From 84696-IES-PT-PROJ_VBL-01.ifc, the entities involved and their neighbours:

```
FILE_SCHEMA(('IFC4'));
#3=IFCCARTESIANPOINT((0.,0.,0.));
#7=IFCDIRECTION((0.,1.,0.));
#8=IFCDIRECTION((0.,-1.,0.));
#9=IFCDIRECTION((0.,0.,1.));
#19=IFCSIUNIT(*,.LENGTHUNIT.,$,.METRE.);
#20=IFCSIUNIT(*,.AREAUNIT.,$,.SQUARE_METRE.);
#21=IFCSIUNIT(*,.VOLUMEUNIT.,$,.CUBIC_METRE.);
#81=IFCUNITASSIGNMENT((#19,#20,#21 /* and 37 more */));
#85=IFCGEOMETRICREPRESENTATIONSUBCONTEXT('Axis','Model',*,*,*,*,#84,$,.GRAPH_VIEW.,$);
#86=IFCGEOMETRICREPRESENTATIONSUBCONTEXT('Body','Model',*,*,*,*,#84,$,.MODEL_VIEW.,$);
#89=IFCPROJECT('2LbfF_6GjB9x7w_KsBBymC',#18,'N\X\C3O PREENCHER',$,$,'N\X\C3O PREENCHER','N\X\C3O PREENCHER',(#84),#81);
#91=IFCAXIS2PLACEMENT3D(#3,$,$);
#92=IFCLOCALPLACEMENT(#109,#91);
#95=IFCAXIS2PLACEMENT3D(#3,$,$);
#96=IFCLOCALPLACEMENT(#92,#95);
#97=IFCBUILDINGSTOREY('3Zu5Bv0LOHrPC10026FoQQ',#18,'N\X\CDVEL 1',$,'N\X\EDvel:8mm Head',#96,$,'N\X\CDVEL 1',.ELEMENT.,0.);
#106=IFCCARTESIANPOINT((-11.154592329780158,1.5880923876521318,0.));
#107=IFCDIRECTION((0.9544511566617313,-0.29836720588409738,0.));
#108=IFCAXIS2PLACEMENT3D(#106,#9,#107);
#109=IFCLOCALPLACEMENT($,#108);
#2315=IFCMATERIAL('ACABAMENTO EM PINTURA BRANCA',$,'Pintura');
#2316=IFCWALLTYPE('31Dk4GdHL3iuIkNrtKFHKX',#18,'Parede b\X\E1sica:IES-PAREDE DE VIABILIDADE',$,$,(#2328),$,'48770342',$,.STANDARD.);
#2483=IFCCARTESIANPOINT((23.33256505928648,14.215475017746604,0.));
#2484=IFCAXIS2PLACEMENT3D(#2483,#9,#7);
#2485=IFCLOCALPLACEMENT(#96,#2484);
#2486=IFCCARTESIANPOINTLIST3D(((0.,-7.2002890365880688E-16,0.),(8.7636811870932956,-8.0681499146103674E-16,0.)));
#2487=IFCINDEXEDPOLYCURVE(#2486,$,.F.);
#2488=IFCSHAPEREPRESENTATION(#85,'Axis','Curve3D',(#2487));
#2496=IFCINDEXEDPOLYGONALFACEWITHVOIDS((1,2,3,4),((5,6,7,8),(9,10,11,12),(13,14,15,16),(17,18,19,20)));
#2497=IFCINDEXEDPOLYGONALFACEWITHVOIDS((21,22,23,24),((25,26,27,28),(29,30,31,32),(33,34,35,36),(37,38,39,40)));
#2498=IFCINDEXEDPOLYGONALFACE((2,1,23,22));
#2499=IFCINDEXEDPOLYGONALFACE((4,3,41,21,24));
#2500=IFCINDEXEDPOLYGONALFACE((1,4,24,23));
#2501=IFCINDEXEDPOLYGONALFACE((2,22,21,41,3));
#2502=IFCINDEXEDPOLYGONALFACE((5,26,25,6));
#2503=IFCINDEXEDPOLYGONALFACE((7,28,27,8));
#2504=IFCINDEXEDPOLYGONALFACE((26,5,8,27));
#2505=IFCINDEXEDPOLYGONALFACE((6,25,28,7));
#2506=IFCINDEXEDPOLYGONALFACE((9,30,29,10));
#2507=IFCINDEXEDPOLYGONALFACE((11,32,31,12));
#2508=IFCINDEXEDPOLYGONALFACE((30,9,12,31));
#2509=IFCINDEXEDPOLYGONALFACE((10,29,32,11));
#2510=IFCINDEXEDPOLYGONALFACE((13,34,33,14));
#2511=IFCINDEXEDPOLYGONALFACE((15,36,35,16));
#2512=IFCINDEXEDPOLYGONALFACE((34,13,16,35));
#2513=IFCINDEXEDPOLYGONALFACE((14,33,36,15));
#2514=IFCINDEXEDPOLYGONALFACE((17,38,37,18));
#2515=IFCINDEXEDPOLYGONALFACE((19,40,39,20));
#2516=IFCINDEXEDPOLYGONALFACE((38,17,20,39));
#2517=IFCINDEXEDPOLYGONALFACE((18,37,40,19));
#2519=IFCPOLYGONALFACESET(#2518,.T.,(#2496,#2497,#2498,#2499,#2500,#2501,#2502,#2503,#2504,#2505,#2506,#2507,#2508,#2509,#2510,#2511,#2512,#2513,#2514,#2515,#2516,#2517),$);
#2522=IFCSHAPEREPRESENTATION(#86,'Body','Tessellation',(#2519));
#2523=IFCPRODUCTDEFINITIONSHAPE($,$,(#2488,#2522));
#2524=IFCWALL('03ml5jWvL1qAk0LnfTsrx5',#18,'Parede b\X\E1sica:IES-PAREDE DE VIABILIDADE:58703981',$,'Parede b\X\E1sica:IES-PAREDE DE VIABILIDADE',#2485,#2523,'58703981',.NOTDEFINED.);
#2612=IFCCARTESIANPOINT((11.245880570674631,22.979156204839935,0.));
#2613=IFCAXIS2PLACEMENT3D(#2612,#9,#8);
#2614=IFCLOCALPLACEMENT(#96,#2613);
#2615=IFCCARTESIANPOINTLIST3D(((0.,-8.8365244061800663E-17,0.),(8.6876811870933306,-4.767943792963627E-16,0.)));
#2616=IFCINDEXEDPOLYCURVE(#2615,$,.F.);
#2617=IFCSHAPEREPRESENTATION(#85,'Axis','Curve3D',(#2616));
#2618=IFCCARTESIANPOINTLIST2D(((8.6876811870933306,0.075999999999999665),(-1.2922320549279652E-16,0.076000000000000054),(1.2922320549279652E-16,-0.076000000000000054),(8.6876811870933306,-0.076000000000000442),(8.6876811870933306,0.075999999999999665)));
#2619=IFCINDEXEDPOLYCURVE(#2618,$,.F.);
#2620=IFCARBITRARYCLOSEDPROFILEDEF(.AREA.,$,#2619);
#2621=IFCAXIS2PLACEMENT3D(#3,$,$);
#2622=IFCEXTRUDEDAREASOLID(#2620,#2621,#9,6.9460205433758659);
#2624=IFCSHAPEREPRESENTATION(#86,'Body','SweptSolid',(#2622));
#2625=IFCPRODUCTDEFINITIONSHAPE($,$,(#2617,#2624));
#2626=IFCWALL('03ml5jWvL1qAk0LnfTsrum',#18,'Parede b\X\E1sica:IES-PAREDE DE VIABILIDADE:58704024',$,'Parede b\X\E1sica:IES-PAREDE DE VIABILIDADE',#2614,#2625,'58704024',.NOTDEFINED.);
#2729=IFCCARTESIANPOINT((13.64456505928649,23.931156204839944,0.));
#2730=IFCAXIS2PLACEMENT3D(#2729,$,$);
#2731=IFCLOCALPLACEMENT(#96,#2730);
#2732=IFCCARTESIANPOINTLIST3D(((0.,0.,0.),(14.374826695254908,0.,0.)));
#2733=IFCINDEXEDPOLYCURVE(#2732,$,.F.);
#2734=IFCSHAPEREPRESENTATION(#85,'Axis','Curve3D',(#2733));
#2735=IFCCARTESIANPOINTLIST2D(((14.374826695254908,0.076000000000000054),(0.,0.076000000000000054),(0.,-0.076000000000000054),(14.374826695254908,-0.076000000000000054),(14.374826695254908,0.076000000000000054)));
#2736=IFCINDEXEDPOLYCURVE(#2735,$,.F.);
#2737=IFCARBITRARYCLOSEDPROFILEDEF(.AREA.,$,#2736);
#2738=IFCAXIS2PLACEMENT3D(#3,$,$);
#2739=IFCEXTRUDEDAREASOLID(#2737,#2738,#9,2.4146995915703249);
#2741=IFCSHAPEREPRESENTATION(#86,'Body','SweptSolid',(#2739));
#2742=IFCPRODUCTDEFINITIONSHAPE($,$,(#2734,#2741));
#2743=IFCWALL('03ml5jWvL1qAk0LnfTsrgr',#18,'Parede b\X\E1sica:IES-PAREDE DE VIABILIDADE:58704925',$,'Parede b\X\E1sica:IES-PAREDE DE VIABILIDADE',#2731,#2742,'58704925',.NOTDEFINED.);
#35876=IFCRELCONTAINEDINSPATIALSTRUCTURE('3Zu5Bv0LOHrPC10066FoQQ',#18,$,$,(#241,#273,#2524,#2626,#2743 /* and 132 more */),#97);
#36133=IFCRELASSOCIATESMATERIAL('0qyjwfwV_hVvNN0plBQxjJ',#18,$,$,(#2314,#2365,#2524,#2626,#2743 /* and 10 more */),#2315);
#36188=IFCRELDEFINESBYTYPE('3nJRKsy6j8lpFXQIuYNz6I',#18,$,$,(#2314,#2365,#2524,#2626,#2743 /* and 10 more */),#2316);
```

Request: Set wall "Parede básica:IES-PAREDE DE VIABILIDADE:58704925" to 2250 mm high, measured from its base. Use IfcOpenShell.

```python
import ifcopenshell
import ifcopenshell.geom
import ifcopenshell.util.representation
import ifcopenshell.util.shape
import ifcopenshell.util.unit

model = ifcopenshell.open("84696-IES-PT-PROJ_VBL-01.ifc")
unit_scale = ifcopenshell.util.unit.calculate_unit_scale(model)
settings = ifcopenshell.geom.settings()


def volume(element):
    """Net volume in cubic metres, openings subtracted."""
    shape = ifcopenshell.geom.create_shape(settings, element)
    return ifcopenshell.util.shape.get_volume(shape.geometry)


wall = model.by_guid("03ml5jWvL1qAk0LnfTsrgr")
before = volume(wall)

body = ifcopenshell.util.representation.get_representation(wall, "Model", "Body")
solid = body.Items[0]
old_height = solid.Depth
solid.Depth = 2.25 / unit_scale
after = volume(wall)

print(f"height {old_height:g} -> {solid.Depth:g}, volume {before:.3f} -> {after:.3f} m3")

model.write("84696-IES-PT-PROJ_VBL-01_updated.ifc")
```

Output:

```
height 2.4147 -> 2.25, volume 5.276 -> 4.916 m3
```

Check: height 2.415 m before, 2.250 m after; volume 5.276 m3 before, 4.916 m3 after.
